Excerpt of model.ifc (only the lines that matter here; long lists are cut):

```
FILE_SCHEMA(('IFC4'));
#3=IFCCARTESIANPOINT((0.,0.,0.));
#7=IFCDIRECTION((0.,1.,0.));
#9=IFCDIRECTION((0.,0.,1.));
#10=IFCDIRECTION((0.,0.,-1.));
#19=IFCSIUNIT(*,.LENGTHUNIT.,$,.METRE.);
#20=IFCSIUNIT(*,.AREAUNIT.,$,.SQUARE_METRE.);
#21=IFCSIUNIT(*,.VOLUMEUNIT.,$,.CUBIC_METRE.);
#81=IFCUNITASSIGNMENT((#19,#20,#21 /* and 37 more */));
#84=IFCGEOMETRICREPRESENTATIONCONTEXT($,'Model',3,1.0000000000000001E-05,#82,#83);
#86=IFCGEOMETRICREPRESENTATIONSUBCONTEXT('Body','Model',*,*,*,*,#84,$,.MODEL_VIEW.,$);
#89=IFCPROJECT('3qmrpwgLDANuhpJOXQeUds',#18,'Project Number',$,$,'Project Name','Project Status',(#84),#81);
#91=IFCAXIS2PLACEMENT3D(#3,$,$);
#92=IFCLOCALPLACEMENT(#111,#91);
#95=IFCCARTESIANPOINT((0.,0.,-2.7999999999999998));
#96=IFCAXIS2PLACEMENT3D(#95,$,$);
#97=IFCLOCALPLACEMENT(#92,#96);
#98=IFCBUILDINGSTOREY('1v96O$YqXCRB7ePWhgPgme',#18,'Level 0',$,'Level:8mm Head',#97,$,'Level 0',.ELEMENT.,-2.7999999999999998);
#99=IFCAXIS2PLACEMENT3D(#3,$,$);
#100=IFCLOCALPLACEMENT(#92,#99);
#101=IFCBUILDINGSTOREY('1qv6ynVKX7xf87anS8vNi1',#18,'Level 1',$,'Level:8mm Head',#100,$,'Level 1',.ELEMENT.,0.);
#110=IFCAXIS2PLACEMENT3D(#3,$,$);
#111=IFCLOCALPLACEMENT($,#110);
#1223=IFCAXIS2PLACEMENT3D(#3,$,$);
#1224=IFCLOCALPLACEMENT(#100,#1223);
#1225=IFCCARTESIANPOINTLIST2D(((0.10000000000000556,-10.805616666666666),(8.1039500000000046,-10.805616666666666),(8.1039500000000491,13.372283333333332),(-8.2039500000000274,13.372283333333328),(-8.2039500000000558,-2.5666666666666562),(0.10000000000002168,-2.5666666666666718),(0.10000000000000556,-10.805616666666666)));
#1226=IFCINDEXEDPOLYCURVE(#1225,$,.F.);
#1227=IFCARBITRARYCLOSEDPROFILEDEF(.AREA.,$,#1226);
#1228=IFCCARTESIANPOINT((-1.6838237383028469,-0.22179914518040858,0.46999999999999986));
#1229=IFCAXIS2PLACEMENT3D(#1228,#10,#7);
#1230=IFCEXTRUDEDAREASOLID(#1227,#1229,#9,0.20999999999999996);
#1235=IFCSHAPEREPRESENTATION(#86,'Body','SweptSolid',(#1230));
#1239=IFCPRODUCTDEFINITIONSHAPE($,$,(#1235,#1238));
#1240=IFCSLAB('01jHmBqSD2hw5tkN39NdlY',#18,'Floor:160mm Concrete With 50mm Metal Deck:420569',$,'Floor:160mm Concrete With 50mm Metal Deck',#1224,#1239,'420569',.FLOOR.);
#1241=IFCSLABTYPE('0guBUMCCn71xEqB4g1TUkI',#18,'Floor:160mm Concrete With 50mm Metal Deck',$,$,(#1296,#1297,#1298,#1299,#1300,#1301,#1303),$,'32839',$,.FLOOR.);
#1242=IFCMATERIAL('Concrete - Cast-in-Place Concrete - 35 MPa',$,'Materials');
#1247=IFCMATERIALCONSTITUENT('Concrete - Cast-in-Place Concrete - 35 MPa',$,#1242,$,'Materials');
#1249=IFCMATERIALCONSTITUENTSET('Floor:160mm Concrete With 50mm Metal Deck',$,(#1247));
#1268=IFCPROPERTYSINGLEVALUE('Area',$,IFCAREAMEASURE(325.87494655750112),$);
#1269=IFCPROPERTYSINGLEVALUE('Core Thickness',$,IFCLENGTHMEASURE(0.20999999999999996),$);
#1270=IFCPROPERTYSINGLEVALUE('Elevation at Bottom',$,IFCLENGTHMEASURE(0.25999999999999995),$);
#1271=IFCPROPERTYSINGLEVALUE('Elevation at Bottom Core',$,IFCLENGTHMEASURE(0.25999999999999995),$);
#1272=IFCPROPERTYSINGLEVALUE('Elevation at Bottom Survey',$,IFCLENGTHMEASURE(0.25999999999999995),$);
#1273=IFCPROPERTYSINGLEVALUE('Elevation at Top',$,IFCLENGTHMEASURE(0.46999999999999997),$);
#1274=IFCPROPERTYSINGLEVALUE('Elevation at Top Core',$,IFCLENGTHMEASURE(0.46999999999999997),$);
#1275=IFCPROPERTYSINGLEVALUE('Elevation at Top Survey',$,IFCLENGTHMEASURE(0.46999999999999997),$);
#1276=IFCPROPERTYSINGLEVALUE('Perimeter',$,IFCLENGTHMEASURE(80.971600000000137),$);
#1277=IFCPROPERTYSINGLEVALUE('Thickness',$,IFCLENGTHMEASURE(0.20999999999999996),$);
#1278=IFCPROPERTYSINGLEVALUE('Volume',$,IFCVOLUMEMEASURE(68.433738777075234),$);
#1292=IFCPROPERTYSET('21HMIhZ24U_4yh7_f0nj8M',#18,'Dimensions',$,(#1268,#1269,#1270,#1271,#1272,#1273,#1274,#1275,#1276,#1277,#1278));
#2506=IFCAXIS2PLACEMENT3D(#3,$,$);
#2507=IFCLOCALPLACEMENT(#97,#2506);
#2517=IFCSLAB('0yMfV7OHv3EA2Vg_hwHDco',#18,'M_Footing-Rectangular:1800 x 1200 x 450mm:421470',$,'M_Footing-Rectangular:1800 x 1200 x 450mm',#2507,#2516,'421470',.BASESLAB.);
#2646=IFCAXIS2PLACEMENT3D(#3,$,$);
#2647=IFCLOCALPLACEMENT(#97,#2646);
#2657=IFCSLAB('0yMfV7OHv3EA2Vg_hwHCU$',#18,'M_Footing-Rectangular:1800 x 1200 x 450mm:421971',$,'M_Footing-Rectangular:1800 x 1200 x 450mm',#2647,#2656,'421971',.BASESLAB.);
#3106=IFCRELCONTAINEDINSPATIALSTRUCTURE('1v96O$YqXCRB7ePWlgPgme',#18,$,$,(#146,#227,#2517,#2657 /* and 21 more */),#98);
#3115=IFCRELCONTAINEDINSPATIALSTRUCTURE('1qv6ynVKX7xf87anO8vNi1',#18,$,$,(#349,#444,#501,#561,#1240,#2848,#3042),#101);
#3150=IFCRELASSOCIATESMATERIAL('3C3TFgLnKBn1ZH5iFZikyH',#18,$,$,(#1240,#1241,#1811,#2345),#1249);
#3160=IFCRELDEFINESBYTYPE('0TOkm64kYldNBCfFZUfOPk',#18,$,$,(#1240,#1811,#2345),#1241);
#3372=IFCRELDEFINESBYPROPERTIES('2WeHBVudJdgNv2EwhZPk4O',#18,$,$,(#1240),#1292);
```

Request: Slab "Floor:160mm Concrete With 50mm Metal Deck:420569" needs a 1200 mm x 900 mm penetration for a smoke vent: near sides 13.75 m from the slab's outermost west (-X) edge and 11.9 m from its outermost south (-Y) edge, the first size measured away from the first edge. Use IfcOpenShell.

```python
import numpy as np
import ifcopenshell
import ifcopenshell.api.feature
import ifcopenshell.api.geometry
import ifcopenshell.api.pset
import ifcopenshell.api.root
import ifcopenshell.geom
import ifcopenshell.util.element
import ifcopenshell.util.placement
import ifcopenshell.util.representation
import ifcopenshell.util.shape
import ifcopenshell.util.unit

model = ifcopenshell.open("model.ifc")
unit_scale = ifcopenshell.util.unit.calculate_unit_scale(model)
area_scale = ifcopenshell.util.unit.calculate_unit_scale(model, "AREAUNIT")
volume_scale = ifcopenshell.util.unit.calculate_unit_scale(model, "VOLUMEUNIT")
settings = ifcopenshell.geom.settings()


def volume(element):
    """Net volume in cubic metres, openings subtracted."""
    shape = ifcopenshell.geom.create_shape(settings, element)
    return ifcopenshell.util.shape.get_volume(shape.geometry)


slab = model.by_guid("01jHmBqSD2hw5tkN39NdlY")
before = volume(slab)

# Extent in the slab's own axes, in metres. The edges named are its -X and -Y sides.
slab_shape = ifcopenshell.geom.create_shape(settings, slab)
vertices = ifcopenshell.util.shape.get_vertices(slab_shape.geometry)
x_min, y_min, bottom = vertices.min(axis=0)
top = vertices[:, 2].max()

opening = ifcopenshell.api.root.create_entity(model, ifc_class="IfcOpeningElement", name="Smoke vent opening", predefined_type="OPENING")
context = ifcopenshell.util.representation.get_context(model, "Model", "Body", "MODEL_VIEW")
width, depth = 1.2, 0.9
outline = [(0.0, 0.0), (width, 0.0), (width, depth), (0.0, depth), (0.0, 0.0)]
# Overshoot both faces by 50 mm so the cut is clean.
shape = ifcopenshell.api.geometry.add_slab_representation(
    model, context=context, depth=top - bottom + 0.1, polyline=outline
)
ifcopenshell.api.geometry.assign_representation(model, product=opening, representation=shape)

matrix = ifcopenshell.util.placement.get_local_placement(slab.ObjectPlacement)
matrix[:, 3] = matrix @ np.append(np.array([x_min + 13.75, y_min + 11.9, bottom - 0.05]) / unit_scale, 1.0)
ifcopenshell.api.geometry.edit_object_placement(model, product=opening, matrix=matrix, is_si=False)
ifcopenshell.api.feature.add_feature(model, feature=opening, element=slab)

after = volume(slab)

# Update the slab's stored quantities.
pset = model.by_id(ifcopenshell.util.element.get_pset(slab, "Dimensions", should_inherit=False)["id"])
ifcopenshell.api.pset.edit_pset(model, pset=pset, properties={
    "Area": model.create_entity("IfcAreaMeasure", after / (top - bottom) / area_scale),
    "Volume": model.create_entity("IfcVolumeMeasure", after / volume_scale),
})

print(f"slab volume {before:.3f} -> {after:.3f} m3")

model.write("model_edited.ifc")
```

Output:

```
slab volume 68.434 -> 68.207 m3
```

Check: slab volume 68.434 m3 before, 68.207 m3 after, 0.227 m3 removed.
